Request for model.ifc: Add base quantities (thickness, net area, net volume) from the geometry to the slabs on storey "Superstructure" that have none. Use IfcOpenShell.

First a look at what the model holds.

```python
import ifcopenshell
import ifcopenshell.util.element
import ifcopenshell.util.unit

model = ifcopenshell.open("model.ifc")
print(model.schema)
for unit_type in ("LENGTHUNIT", "AREAUNIT", "VOLUMEUNIT"):
    print(unit_type, ifcopenshell.util.unit.calculate_unit_scale(model, unit_type))
storey = next(s for s in model.by_type("IfcBuildingStorey") if s.Name == "Superstructure")
slabs = [e for e in ifcopenshell.util.element.get_decomposition(storey) if e.is_a("IfcSlab")]
for e in sorted(slabs, key=lambda e: e.id()):
    print(e.id(), e.is_a(), e.Name, list(ifcopenshell.util.element.get_psets(e, qtos_only=True)), sep=" | ")
```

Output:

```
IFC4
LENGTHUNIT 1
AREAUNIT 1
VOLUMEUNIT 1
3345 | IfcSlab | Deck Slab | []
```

```python
import ifcopenshell
import ifcopenshell.api.pset
import ifcopenshell.geom
import ifcopenshell.util.element
import ifcopenshell.util.shape
import ifcopenshell.util.unit

model = ifcopenshell.open("model.ifc")
unit_scale = ifcopenshell.util.unit.calculate_unit_scale(model)
area_scale = ifcopenshell.util.unit.calculate_unit_scale(model, "AREAUNIT")
volume_scale = ifcopenshell.util.unit.calculate_unit_scale(model, "VOLUMEUNIT")
settings = ifcopenshell.geom.settings()

storey = next(s for s in model.by_type("IfcBuildingStorey") if s.Name == "Superstructure")
slabs = [e for e in ifcopenshell.util.element.get_decomposition(storey) if e.is_a("IfcSlab")]

for e in sorted(slabs, key=lambda e: e.id()):
    if ifcopenshell.util.element.get_psets(e, qtos_only=True, should_inherit=False):
        continue
    # Geometry comes back in metres, in the element's own axes.
    shape = ifcopenshell.geom.create_shape(settings, e)
    values = {
        "Width": ifcopenshell.util.shape.get_z(shape.geometry) / unit_scale,
        "NetArea": ifcopenshell.util.shape.get_footprint_area(shape.geometry) / area_scale,
        "NetVolume": ifcopenshell.util.shape.get_volume(shape.geometry) / volume_scale,
    }
    qto = ifcopenshell.api.pset.add_qto(model, product=e, name="Qto_SlabBaseQuantities")
    ifcopenshell.api.pset.edit_qto(model, qto=qto, properties=values)
    print(e.id(), {k: round(v, 3) for k, v in values.items()})

model.write("model_updated.ifc")
```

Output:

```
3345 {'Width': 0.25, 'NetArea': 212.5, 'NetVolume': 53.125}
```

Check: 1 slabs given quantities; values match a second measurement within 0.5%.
